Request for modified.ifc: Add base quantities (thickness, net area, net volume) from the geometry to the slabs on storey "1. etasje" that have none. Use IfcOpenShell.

First a look at what the model holds.

```python
import ifcopenshell
import ifcopenshell.util.element
import ifcopenshell.util.unit

model = ifcopenshell.open("modified.ifc")
print(model.schema)
for unit_type in ("LENGTHUNIT", "AREAUNIT", "VOLUMEUNIT"):
    print(unit_type, ifcopenshell.util.unit.calculate_unit_scale(model, unit_type))
storey = next(s for s in model.by_type("IfcBuildingStorey") if s.Name == "1. etasje")
slabs = [e for e in ifcopenshell.util.element.get_decomposition(storey) if e.is_a("IfcSlab")]
for e in sorted(slabs, key=lambda e: e.id()):
    print(e.id(), e.is_a(), e.Name, list(ifcopenshell.util.element.get_psets(e, qtos_only=True)), sep=" | ")
```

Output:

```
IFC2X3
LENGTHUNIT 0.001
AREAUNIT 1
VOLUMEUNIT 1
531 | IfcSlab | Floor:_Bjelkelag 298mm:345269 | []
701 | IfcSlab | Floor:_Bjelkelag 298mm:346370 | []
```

```python
import ifcopenshell
import ifcopenshell.api.pset
import ifcopenshell.geom
import ifcopenshell.util.element
import ifcopenshell.util.shape
import ifcopenshell.util.unit

model = ifcopenshell.open("modified.ifc")
unit_scale = ifcopenshell.util.unit.calculate_unit_scale(model)
area_scale = ifcopenshell.util.unit.calculate_unit_scale(model, "AREAUNIT")
volume_scale = ifcopenshell.util.unit.calculate_unit_scale(model, "VOLUMEUNIT")
settings = ifcopenshell.geom.settings()

storey = next(s for s in model.by_type("IfcBuildingStorey") if s.Name == "1. etasje")
slabs = [e for e in ifcopenshell.util.element.get_decomposition(storey) if e.is_a("IfcSlab")]

for e in sorted(slabs, key=lambda e: e.id()):
    if ifcopenshell.util.element.get_psets(e, qtos_only=True, should_inherit=False):
        continue
    # Geometry comes back in metres, in the element's own axes.
    shape = ifcopenshell.geom.create_shape(settings, e)
    values = {
        "Width": ifcopenshell.util.shape.get_z(shape.geometry) / unit_scale,
        "NetArea": ifcopenshell.util.shape.get_footprint_area(shape.geometry) / area_scale,
        "NetVolume": ifcopenshell.util.shape.get_volume(shape.geometry) / volume_scale,
    }
    qto = ifcopenshell.api.pset.add_qto(model, product=e, name="BaseQuantities")
    ifcopenshell.api.pset.edit_qto(model, qto=qto, properties=values)
    print(e.id(), {k: round(v, 3) for k, v in values.items()})

model.write("modified_edited.ifc")
```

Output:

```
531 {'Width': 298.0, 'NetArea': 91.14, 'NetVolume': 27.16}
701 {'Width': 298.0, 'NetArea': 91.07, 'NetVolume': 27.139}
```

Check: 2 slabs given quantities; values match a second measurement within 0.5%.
